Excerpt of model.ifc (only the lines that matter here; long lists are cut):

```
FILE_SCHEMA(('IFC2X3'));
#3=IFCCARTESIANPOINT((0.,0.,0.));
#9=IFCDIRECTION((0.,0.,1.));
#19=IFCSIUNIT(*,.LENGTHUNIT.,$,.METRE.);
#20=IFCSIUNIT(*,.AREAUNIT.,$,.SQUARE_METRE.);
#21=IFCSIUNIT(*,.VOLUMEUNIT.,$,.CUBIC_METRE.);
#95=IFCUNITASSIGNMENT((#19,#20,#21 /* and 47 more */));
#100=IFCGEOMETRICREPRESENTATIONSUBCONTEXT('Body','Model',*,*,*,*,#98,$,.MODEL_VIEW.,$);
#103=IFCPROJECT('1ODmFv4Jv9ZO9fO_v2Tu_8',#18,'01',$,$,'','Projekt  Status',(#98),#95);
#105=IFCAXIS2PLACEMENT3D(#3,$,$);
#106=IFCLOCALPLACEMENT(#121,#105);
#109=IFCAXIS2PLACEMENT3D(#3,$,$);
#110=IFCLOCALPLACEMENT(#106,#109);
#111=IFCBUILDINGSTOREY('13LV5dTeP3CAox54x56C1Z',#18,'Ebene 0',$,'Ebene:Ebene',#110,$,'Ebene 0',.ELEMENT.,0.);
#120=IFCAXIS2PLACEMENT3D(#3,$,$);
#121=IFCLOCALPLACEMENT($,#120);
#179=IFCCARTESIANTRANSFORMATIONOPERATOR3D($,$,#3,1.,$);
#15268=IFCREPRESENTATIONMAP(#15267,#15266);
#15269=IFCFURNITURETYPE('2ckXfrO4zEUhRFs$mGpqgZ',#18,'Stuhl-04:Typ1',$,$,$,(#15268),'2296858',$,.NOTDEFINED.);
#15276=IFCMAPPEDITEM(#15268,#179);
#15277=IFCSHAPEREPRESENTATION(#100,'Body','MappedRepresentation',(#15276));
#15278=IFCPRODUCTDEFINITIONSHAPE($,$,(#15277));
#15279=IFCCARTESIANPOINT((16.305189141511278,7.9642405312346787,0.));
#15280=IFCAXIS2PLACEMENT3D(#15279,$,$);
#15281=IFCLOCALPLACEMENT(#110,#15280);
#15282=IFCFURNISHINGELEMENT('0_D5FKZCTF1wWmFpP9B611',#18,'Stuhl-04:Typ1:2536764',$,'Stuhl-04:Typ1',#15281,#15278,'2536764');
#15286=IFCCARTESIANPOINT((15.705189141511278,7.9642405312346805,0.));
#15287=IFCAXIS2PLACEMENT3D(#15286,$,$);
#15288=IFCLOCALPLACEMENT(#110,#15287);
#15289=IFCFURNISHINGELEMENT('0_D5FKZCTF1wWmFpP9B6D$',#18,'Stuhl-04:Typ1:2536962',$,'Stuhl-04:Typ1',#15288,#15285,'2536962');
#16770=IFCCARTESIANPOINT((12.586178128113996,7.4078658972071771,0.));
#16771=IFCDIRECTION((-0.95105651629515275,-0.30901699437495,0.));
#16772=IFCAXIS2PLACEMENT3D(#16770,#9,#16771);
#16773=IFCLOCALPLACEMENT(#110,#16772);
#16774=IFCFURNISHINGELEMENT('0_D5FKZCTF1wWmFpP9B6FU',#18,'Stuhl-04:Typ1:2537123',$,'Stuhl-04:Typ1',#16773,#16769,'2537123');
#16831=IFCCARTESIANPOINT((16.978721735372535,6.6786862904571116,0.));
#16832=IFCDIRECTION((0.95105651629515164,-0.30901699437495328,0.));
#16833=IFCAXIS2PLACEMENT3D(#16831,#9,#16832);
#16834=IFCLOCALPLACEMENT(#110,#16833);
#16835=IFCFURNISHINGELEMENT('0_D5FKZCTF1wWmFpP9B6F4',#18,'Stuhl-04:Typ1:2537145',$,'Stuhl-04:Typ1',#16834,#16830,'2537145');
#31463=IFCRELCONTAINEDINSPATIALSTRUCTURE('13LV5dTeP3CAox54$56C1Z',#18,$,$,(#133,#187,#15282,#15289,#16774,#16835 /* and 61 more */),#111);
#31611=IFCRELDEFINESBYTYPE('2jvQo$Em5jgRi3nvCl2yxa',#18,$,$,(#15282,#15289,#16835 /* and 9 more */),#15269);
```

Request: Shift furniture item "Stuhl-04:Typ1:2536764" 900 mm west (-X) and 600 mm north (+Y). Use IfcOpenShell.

```python
import ifcopenshell
import ifcopenshell.api.geometry
import ifcopenshell.util.placement

model = ifcopenshell.open("model.ifc")

item = model.by_guid("0_D5FKZCTF1wWmFpP9B611")
matrix = ifcopenshell.util.placement.get_local_placement(item.ObjectPlacement)
matrix[0, 3] -= 0.9
matrix[1, 3] += 0.6
ifcopenshell.api.geometry.edit_object_placement(model, product=item, matrix=matrix, is_si=False)

print(ifcopenshell.util.placement.get_local_placement(item.ObjectPlacement).round(3) + 0.0)

model.write("model_edited.ifc")
```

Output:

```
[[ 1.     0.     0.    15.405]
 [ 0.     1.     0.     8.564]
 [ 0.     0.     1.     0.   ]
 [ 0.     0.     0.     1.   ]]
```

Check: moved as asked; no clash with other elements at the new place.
